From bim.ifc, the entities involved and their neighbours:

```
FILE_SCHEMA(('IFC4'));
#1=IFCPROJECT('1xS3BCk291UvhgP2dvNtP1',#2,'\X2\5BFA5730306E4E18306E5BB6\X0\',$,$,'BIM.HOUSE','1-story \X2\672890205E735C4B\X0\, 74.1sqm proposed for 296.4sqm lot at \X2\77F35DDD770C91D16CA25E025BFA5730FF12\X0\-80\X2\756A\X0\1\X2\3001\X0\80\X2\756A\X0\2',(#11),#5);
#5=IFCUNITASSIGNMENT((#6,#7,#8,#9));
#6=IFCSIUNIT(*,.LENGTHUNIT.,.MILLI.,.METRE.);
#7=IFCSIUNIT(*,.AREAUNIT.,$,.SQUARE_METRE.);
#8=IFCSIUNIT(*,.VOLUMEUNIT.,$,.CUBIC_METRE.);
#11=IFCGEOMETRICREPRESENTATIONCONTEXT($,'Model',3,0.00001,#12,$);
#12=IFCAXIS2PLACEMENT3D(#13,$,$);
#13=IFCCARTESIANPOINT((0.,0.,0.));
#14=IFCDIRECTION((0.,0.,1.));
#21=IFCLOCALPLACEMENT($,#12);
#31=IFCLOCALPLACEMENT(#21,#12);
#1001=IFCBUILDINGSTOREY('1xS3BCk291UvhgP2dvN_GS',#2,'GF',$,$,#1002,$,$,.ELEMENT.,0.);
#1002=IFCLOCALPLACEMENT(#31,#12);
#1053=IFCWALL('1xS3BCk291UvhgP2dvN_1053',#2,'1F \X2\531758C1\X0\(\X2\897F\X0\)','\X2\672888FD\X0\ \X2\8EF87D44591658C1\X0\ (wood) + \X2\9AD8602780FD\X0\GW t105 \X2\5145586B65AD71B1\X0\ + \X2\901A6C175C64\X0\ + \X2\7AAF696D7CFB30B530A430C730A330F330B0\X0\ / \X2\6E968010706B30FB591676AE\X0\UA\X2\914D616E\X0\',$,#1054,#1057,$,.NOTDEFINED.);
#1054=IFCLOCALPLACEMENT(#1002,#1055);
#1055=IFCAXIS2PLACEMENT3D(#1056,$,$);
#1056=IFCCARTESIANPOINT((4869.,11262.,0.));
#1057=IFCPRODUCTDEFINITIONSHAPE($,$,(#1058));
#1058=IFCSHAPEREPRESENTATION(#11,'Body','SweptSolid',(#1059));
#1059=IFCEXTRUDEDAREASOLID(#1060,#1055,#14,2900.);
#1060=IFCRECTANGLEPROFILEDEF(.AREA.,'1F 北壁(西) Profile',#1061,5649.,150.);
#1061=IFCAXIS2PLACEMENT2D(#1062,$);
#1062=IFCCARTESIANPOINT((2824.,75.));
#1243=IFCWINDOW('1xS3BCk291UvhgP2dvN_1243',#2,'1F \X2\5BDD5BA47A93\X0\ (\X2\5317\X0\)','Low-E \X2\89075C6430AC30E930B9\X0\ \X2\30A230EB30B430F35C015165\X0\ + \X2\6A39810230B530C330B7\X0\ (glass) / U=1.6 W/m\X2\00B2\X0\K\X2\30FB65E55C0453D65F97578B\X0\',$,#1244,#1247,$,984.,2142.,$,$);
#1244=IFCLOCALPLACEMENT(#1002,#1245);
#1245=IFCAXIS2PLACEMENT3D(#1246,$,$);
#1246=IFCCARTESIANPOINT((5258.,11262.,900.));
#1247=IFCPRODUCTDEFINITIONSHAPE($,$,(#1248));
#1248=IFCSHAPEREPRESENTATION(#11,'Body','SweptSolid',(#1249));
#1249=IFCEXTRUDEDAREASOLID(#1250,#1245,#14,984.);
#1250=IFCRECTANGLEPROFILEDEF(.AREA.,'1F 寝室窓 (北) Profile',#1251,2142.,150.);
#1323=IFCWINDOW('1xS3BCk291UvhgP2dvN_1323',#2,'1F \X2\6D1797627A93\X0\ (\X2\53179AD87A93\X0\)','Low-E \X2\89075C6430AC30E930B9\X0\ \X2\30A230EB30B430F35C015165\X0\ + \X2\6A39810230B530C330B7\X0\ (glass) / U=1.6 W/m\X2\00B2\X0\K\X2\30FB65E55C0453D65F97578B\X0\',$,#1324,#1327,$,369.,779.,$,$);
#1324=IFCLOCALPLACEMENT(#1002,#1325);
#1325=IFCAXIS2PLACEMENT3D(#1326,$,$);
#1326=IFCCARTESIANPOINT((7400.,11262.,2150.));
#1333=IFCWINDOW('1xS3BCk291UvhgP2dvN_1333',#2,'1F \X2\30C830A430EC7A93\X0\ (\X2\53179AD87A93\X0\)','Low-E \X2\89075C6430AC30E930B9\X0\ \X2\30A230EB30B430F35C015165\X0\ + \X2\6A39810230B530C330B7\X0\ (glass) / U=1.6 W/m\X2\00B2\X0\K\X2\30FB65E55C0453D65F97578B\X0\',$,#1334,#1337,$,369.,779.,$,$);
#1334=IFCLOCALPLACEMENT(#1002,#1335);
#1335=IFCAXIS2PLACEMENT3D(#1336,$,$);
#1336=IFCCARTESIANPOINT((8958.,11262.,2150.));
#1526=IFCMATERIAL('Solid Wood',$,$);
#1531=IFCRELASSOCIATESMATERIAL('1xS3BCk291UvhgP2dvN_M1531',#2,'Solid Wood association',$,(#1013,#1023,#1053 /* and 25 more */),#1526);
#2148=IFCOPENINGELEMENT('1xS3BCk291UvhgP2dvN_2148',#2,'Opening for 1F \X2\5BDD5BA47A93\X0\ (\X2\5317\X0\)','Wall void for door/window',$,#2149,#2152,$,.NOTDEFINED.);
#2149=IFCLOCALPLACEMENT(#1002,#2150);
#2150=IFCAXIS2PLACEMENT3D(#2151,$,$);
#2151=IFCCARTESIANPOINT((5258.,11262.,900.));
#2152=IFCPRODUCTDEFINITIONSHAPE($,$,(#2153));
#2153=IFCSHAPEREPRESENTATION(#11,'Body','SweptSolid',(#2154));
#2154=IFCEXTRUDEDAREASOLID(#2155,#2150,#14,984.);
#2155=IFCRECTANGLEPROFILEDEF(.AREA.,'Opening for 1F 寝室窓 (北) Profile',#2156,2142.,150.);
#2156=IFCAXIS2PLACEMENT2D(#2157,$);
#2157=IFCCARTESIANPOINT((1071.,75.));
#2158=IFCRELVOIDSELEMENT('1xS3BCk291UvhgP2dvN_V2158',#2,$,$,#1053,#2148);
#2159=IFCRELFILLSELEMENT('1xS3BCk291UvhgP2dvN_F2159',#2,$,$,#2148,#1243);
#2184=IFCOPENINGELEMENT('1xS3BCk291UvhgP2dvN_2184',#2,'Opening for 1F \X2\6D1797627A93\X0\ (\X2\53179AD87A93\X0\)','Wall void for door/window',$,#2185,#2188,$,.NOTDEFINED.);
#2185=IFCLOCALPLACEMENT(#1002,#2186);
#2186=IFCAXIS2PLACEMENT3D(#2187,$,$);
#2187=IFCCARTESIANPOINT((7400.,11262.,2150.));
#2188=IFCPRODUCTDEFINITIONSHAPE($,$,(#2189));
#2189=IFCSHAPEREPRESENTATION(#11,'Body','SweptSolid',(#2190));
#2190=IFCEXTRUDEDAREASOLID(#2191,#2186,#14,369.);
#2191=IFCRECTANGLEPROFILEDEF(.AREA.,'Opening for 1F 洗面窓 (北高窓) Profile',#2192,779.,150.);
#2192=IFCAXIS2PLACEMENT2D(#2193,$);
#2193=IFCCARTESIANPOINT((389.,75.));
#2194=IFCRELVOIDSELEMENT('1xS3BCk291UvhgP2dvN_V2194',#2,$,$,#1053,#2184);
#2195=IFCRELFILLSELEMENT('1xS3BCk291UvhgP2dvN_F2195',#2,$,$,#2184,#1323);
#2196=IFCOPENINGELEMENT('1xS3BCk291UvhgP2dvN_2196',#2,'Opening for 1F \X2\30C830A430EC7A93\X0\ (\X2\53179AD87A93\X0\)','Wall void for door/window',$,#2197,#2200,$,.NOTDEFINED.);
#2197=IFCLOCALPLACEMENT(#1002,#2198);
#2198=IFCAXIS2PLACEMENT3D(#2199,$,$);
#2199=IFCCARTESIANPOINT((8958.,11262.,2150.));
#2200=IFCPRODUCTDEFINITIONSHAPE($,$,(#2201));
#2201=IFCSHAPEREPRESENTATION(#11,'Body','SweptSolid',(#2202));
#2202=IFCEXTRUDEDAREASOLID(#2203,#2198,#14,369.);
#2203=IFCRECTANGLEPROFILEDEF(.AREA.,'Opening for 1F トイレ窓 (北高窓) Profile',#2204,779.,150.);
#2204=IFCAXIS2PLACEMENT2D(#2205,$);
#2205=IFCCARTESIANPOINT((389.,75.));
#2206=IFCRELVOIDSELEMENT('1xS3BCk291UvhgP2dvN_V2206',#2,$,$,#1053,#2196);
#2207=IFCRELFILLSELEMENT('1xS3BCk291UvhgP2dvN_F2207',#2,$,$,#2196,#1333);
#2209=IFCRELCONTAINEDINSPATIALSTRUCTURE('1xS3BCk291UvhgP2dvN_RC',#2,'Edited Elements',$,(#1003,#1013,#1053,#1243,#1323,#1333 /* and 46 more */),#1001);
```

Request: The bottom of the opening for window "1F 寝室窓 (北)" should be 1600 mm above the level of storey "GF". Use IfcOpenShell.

```python
import numpy as np
import ifcopenshell
import ifcopenshell.api.geometry
import ifcopenshell.geom
import ifcopenshell.util.element
import ifcopenshell.util.placement
import ifcopenshell.util.shape
import ifcopenshell.util.unit

model = ifcopenshell.open("bim.ifc")
unit_scale = ifcopenshell.util.unit.calculate_unit_scale(model)

window = model.by_guid("1xS3BCk291UvhgP2dvN_1243")
opening = window.FillsVoids[0].RelatingOpeningElement
storey = ifcopenshell.util.element.get_container(window, ifc_class="IfcBuildingStorey")
level = ifcopenshell.util.placement.get_local_placement(storey.ObjectPlacement)[2, 3]

# The opening's origin need not be at the sill, so measure its lowest point.
shape = ifcopenshell.geom.create_shape(ifcopenshell.geom.settings(), opening)
bottom = ifcopenshell.util.shape.get_shape_bottom_elevation(shape, shape.geometry) / unit_scale
dz = level + 1.6 / unit_scale - bottom

shift = np.array([0.0, 0.0, dz])
# The window is not placed relative to its opening, so move both.
for product in (opening, window):
    matrix = ifcopenshell.util.placement.get_local_placement(product.ObjectPlacement)
    matrix[:3, 3] += shift
    ifcopenshell.api.geometry.edit_object_placement(model, product=product, matrix=matrix, is_si=False)

print(f"moved by {dz * unit_scale:+.3f} m")

model.write("bim-out.ifc")
```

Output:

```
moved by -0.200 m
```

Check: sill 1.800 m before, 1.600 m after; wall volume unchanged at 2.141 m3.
